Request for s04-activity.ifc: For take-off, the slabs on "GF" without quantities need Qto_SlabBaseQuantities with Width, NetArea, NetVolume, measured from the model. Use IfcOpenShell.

First a look at what the model holds.

```python
import ifcopenshell
import ifcopenshell.util.element
import ifcopenshell.util.unit

model = ifcopenshell.open("s04-activity.ifc")
print(model.schema)
for unit_type in ("LENGTHUNIT", "AREAUNIT", "VOLUMEUNIT"):
    print(unit_type, ifcopenshell.util.unit.calculate_unit_scale(model, unit_type))
storey = next(s for s in model.by_type("IfcBuildingStorey") if s.Name == "GF")
slabs = [e for e in ifcopenshell.util.element.get_decomposition(storey) if e.is_a("IfcSlab")]
for e in sorted(slabs, key=lambda e: e.id()):
    print(e.id(), e.is_a(), e.Name, list(ifcopenshell.util.element.get_psets(e, qtos_only=True)), sep=" | ")
```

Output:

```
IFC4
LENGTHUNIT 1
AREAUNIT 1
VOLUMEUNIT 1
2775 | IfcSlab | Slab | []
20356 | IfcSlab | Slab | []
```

```python
import ifcopenshell
import ifcopenshell.api.pset
import ifcopenshell.geom
import ifcopenshell.util.element
import ifcopenshell.util.shape
import ifcopenshell.util.unit

model = ifcopenshell.open("s04-activity.ifc")
unit_scale = ifcopenshell.util.unit.calculate_unit_scale(model)
area_scale = ifcopenshell.util.unit.calculate_unit_scale(model, "AREAUNIT")
volume_scale = ifcopenshell.util.unit.calculate_unit_scale(model, "VOLUMEUNIT")
settings = ifcopenshell.geom.settings()

storey = next(s for s in model.by_type("IfcBuildingStorey") if s.Name == "GF")
slabs = [e for e in ifcopenshell.util.element.get_decomposition(storey) if e.is_a("IfcSlab")]

for e in sorted(slabs, key=lambda e: e.id()):
    if ifcopenshell.util.element.get_psets(e, qtos_only=True, should_inherit=False):
        continue
    # Geometry comes back in metres, in the element's own axes.
    shape = ifcopenshell.geom.create_shape(settings, e)
    values = {
        "Width": ifcopenshell.util.shape.get_z(shape.geometry) / unit_scale,
        "NetArea": ifcopenshell.util.shape.get_footprint_area(shape.geometry) / area_scale,
        "NetVolume": ifcopenshell.util.shape.get_volume(shape.geometry) / volume_scale,
    }
    qto = ifcopenshell.api.pset.add_qto(model, product=e, name="Qto_SlabBaseQuantities")
    ifcopenshell.api.pset.edit_qto(model, qto=qto, properties=values)
    print(e.id(), {k: round(v, 3) for k, v in values.items()})

model.write("s04-activity_rev.ifc")
```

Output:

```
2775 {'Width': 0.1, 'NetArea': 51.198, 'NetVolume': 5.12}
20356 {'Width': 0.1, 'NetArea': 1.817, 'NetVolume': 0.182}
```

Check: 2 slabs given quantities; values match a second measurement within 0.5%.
